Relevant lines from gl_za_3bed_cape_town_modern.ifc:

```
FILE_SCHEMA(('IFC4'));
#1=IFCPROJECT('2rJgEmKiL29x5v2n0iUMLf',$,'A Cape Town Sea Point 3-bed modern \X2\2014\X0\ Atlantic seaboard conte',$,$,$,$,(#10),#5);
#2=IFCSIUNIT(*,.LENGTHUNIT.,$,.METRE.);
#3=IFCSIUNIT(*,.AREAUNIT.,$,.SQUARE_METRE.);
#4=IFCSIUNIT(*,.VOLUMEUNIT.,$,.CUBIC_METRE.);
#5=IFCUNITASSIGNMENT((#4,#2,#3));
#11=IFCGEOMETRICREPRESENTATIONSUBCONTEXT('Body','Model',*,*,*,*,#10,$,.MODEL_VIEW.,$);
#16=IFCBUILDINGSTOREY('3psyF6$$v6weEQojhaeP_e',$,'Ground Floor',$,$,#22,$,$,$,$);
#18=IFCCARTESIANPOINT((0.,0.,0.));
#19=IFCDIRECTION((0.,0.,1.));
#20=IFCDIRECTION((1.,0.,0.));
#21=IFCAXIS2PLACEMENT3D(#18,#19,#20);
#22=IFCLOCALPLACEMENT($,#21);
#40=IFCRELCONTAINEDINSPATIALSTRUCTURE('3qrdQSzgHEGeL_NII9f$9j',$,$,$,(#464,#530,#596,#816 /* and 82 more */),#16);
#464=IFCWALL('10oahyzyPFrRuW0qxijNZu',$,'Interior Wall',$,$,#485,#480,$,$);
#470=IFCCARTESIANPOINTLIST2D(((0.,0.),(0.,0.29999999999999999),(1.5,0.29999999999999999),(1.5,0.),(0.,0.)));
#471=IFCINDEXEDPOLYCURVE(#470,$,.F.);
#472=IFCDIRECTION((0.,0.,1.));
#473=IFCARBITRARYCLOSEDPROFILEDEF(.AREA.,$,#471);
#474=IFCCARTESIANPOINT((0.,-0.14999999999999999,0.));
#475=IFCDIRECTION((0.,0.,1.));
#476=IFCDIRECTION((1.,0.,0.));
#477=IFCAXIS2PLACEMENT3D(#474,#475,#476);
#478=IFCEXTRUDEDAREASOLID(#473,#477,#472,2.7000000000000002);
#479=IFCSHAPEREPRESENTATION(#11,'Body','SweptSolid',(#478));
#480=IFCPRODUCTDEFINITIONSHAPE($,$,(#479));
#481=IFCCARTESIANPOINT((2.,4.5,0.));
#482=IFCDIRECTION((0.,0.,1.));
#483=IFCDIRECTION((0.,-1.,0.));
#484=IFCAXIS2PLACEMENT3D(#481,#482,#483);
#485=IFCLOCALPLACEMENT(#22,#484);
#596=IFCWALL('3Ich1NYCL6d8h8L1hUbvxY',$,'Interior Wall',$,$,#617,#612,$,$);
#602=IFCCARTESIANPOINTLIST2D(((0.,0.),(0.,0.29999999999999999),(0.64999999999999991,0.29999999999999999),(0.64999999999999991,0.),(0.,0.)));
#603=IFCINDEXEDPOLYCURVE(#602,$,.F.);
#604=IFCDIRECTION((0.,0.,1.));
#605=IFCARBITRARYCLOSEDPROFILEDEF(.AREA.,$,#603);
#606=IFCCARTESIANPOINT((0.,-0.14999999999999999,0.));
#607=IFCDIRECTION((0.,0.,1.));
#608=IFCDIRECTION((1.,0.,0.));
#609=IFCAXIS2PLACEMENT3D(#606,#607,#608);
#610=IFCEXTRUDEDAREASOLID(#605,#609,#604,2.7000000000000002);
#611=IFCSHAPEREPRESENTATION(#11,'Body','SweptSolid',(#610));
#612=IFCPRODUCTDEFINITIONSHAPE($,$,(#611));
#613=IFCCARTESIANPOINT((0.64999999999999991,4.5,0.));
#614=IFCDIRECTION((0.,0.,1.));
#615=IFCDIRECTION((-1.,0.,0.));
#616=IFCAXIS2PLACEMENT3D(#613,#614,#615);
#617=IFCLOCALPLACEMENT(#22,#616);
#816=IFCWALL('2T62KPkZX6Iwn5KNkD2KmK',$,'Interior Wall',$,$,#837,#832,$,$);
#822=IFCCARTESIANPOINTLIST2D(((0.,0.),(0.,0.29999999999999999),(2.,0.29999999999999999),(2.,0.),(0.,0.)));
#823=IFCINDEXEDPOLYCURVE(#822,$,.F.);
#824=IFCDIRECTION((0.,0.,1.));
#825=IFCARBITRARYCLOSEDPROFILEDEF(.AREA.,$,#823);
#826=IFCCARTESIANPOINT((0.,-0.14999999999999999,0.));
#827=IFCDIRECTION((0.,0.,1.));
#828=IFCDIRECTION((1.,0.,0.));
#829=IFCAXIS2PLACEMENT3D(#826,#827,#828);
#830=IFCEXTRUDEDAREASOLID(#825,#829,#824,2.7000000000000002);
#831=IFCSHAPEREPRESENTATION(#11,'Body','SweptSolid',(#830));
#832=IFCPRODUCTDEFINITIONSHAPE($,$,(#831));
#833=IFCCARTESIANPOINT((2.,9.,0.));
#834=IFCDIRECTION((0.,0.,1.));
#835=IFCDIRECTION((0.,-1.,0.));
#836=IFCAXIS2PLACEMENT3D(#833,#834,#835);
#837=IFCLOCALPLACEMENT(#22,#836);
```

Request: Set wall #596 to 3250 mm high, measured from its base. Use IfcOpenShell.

```python
import ifcopenshell
import ifcopenshell.geom
import ifcopenshell.util.representation
import ifcopenshell.util.shape
import ifcopenshell.util.unit

model = ifcopenshell.open("gl_za_3bed_cape_town_modern.ifc")
unit_scale = ifcopenshell.util.unit.calculate_unit_scale(model)
settings = ifcopenshell.geom.settings()


def volume(element):
    """Net volume in cubic metres, openings subtracted."""
    shape = ifcopenshell.geom.create_shape(settings, element)
    return ifcopenshell.util.shape.get_volume(shape.geometry)


wall = model.by_guid("3Ich1NYCL6d8h8L1hUbvxY")
before = volume(wall)

body = ifcopenshell.util.representation.get_representation(wall, "Model", "Body")
solid = body.Items[0]
old_height = solid.Depth
solid.Depth = 3.25 / unit_scale
after = volume(wall)

print(f"height {old_height:g} -> {solid.Depth:g}, volume {before:.3f} -> {after:.3f} m3")

model.write("gl_za_3bed_cape_town_modern_rev.ifc")
```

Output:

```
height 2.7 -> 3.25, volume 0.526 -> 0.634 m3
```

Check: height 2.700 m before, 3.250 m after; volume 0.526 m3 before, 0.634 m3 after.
